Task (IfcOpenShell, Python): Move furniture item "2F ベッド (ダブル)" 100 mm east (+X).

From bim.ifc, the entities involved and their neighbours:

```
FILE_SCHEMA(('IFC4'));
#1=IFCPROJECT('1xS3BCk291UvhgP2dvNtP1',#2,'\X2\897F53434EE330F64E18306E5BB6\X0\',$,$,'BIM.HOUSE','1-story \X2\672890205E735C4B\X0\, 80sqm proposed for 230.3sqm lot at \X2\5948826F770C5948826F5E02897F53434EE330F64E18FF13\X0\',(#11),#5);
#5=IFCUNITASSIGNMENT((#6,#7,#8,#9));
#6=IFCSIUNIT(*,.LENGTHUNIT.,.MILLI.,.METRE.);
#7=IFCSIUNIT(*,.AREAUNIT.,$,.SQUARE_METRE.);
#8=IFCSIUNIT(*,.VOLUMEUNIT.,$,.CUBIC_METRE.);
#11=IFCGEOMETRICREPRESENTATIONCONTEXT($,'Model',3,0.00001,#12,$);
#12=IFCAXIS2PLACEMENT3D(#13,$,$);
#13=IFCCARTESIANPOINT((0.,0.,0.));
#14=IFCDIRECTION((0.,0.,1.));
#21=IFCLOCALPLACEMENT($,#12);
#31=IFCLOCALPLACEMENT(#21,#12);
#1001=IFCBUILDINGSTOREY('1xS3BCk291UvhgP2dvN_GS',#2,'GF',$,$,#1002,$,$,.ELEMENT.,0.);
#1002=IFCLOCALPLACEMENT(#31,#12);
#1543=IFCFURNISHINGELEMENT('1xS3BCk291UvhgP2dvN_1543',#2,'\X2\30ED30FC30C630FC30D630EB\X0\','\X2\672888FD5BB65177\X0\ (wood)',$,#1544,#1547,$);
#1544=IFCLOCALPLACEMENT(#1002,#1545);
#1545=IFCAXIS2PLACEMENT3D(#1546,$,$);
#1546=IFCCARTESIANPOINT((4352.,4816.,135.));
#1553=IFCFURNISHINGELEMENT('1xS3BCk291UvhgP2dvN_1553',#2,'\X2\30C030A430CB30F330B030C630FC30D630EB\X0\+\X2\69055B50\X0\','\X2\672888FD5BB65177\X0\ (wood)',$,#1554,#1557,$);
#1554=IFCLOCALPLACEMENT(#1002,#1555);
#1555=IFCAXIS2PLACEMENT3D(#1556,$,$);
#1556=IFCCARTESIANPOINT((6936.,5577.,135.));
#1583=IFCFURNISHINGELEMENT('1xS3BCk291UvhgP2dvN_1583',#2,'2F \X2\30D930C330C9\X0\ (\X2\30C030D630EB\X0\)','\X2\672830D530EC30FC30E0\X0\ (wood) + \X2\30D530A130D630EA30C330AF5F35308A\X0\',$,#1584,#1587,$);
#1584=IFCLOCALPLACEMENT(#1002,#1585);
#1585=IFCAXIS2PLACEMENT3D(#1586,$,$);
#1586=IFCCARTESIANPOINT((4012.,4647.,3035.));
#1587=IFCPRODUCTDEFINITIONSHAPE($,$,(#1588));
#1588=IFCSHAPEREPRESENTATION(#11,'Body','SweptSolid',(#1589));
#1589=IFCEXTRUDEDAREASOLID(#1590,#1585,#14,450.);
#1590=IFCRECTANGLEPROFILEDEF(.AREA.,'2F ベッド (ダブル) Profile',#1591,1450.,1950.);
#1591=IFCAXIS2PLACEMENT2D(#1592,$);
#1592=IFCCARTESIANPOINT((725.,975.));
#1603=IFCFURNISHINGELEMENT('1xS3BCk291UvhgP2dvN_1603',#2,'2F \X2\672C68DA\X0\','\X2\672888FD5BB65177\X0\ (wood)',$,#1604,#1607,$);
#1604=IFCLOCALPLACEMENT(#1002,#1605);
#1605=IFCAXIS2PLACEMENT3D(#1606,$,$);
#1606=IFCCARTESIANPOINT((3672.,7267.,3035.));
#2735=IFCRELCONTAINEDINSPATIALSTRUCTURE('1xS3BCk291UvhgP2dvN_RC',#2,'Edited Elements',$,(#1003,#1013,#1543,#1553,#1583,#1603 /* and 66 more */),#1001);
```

```python
import ifcopenshell
import ifcopenshell.api.geometry
import ifcopenshell.util.placement
import ifcopenshell.util.unit

model = ifcopenshell.open("bim.ifc")
unit_scale = ifcopenshell.util.unit.calculate_unit_scale(model)

item = model.by_guid("1xS3BCk291UvhgP2dvN_1583")
matrix = ifcopenshell.util.placement.get_local_placement(item.ObjectPlacement)
matrix[0, 3] += 0.1 / unit_scale
ifcopenshell.api.geometry.edit_object_placement(model, product=item, matrix=matrix, is_si=False)

print(ifcopenshell.util.placement.get_local_placement(item.ObjectPlacement).round(3) + 0.0)

model.write("bim_updated.ifc")
```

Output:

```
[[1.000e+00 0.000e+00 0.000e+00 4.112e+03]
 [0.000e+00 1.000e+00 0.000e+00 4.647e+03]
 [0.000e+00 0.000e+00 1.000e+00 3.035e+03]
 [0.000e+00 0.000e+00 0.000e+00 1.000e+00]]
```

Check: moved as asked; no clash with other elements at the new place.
